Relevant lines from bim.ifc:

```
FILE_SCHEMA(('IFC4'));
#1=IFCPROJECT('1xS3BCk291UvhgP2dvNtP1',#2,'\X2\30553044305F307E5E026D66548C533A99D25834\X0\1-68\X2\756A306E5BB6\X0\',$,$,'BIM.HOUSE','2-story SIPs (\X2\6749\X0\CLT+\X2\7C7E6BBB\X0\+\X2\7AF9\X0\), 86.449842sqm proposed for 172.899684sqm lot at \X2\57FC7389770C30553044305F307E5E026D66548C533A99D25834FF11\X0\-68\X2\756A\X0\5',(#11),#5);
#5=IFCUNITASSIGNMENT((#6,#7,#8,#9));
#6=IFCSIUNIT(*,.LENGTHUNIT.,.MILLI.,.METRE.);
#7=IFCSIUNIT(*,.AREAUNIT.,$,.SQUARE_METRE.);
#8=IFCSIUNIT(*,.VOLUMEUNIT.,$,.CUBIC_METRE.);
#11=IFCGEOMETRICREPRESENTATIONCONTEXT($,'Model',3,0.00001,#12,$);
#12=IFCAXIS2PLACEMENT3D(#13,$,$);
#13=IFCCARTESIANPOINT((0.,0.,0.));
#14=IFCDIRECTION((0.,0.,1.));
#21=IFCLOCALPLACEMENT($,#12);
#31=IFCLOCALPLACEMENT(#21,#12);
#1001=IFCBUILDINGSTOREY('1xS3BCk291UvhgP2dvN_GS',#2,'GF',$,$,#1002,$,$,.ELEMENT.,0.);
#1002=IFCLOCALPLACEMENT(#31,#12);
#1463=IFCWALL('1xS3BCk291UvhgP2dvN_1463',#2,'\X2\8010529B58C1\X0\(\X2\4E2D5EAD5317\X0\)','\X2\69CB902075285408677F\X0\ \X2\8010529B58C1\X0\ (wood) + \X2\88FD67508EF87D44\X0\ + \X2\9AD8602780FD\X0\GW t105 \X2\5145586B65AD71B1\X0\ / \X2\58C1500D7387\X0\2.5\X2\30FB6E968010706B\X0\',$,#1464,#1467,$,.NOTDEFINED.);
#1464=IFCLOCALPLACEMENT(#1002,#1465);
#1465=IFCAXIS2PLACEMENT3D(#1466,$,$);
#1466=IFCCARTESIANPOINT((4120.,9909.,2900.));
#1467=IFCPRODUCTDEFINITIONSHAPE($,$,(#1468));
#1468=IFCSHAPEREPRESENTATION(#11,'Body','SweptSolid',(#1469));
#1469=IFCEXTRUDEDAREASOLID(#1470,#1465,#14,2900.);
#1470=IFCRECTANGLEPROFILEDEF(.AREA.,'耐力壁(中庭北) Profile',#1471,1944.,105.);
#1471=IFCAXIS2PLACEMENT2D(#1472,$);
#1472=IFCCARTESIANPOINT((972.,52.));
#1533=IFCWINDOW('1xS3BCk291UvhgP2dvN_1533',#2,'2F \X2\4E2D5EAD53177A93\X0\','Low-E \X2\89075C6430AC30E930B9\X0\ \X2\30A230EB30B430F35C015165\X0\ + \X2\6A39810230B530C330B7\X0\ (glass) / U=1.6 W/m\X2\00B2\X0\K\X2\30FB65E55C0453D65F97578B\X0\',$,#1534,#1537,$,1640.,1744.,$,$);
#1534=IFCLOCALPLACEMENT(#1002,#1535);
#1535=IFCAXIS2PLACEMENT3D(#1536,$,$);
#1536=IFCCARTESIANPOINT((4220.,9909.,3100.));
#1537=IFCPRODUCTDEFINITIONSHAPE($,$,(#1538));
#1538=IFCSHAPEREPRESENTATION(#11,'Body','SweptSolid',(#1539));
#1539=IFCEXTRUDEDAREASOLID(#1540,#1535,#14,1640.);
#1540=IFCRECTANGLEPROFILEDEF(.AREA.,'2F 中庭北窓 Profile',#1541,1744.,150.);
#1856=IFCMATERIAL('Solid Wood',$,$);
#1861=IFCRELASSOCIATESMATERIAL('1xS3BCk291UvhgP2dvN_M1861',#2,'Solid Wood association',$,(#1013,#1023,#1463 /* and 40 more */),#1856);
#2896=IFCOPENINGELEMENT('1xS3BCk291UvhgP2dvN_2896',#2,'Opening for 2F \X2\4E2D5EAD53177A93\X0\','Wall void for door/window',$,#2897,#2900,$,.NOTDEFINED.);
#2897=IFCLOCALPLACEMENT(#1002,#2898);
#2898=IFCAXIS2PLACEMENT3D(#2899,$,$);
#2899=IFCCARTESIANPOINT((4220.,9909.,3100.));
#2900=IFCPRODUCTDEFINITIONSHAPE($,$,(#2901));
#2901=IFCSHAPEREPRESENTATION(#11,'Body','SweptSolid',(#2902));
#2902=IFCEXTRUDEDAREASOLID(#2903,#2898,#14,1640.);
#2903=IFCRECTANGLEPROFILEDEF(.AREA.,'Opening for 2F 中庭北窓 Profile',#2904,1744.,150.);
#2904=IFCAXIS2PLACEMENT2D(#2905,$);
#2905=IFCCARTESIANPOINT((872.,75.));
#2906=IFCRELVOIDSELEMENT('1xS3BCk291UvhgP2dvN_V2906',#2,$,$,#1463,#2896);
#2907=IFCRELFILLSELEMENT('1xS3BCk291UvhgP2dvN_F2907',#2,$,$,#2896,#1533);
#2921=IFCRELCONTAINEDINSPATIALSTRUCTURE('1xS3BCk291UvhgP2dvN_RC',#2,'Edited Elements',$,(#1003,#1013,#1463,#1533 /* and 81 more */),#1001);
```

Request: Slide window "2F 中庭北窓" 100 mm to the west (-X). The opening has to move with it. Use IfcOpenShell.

```python
import ifcopenshell
import ifcopenshell.api.geometry
import ifcopenshell.util.placement
import ifcopenshell.util.unit

model = ifcopenshell.open("bim.ifc")
unit_scale = ifcopenshell.util.unit.calculate_unit_scale(model)

window = model.by_guid("1xS3BCk291UvhgP2dvN_1533")
opening = window.FillsVoids[0].RelatingOpeningElement
wall = opening.VoidsElements[0].RelatingBuildingElement

wall_matrix = ifcopenshell.util.placement.get_local_placement(wall.ObjectPlacement)
shift = wall_matrix[:3, 0] * -0.1 / unit_scale
before = ifcopenshell.util.placement.get_local_placement(window.ObjectPlacement)[:3, 3].copy()

# The window is not placed relative to its opening, so move both.
for product in (opening, window):
    matrix = ifcopenshell.util.placement.get_local_placement(product.ObjectPlacement)
    matrix[:3, 3] += shift
    ifcopenshell.api.geometry.edit_object_placement(model, product=product, matrix=matrix, is_si=False)

after = ifcopenshell.util.placement.get_local_placement(window.ObjectPlacement)[:3, 3]
print("window moved by", (after - before).round(3) + 0.0)

model.write("bim-out.ifc")
```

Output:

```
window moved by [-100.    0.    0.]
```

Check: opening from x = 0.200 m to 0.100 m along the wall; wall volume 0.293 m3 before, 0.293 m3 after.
